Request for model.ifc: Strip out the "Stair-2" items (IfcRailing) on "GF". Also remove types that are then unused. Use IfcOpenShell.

First a look at what the model holds.

```python
import ifcopenshell
import ifcopenshell.util.element

model = ifcopenshell.open("model.ifc")
print(model.schema)
storey = next(s for s in model.by_type("IfcBuildingStorey") if s.Name == "GF")
railings = [e for e in ifcopenshell.util.element.get_decomposition(storey) if e.is_a("IfcRailing")]
seen = {}
for e in railings:
    element_type = ifcopenshell.util.element.get_type(e)
    name = element_type.Name if element_type not in (None, e) else None
    seen[name] = seen.get(name, 0) + 1
for name, count in sorted(seen.items(), key=str):
    print(count, "x", name)
```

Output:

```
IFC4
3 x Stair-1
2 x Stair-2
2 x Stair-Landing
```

```python
import ifcopenshell
import ifcopenshell.api.root
import ifcopenshell.util.element

model = ifcopenshell.open("model.ifc")

storey = next(s for s in model.by_type("IfcBuildingStorey") if s.Name == "GF")
railings = [e for e in ifcopenshell.util.element.get_decomposition(storey) if e.is_a("IfcRailing")]
targets = [e for e in railings if (t := ifcopenshell.util.element.get_type(e)) not in (None, e) and t.Name == "Stair-2"]
types = {ifcopenshell.util.element.get_type(e) for e in targets} - {None, *targets}

for e in targets:
    ifcopenshell.api.root.remove_product(model, product=e)
print(len(targets), "removed")

unused = [t for t in types if not ifcopenshell.util.element.get_types(t)]
for t in unused:
    ifcopenshell.api.root.remove_product(model, product=t)
print(len(unused), "unused types removed")

model.write("model_rev.ifc")
```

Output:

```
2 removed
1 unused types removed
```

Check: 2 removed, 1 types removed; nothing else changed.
